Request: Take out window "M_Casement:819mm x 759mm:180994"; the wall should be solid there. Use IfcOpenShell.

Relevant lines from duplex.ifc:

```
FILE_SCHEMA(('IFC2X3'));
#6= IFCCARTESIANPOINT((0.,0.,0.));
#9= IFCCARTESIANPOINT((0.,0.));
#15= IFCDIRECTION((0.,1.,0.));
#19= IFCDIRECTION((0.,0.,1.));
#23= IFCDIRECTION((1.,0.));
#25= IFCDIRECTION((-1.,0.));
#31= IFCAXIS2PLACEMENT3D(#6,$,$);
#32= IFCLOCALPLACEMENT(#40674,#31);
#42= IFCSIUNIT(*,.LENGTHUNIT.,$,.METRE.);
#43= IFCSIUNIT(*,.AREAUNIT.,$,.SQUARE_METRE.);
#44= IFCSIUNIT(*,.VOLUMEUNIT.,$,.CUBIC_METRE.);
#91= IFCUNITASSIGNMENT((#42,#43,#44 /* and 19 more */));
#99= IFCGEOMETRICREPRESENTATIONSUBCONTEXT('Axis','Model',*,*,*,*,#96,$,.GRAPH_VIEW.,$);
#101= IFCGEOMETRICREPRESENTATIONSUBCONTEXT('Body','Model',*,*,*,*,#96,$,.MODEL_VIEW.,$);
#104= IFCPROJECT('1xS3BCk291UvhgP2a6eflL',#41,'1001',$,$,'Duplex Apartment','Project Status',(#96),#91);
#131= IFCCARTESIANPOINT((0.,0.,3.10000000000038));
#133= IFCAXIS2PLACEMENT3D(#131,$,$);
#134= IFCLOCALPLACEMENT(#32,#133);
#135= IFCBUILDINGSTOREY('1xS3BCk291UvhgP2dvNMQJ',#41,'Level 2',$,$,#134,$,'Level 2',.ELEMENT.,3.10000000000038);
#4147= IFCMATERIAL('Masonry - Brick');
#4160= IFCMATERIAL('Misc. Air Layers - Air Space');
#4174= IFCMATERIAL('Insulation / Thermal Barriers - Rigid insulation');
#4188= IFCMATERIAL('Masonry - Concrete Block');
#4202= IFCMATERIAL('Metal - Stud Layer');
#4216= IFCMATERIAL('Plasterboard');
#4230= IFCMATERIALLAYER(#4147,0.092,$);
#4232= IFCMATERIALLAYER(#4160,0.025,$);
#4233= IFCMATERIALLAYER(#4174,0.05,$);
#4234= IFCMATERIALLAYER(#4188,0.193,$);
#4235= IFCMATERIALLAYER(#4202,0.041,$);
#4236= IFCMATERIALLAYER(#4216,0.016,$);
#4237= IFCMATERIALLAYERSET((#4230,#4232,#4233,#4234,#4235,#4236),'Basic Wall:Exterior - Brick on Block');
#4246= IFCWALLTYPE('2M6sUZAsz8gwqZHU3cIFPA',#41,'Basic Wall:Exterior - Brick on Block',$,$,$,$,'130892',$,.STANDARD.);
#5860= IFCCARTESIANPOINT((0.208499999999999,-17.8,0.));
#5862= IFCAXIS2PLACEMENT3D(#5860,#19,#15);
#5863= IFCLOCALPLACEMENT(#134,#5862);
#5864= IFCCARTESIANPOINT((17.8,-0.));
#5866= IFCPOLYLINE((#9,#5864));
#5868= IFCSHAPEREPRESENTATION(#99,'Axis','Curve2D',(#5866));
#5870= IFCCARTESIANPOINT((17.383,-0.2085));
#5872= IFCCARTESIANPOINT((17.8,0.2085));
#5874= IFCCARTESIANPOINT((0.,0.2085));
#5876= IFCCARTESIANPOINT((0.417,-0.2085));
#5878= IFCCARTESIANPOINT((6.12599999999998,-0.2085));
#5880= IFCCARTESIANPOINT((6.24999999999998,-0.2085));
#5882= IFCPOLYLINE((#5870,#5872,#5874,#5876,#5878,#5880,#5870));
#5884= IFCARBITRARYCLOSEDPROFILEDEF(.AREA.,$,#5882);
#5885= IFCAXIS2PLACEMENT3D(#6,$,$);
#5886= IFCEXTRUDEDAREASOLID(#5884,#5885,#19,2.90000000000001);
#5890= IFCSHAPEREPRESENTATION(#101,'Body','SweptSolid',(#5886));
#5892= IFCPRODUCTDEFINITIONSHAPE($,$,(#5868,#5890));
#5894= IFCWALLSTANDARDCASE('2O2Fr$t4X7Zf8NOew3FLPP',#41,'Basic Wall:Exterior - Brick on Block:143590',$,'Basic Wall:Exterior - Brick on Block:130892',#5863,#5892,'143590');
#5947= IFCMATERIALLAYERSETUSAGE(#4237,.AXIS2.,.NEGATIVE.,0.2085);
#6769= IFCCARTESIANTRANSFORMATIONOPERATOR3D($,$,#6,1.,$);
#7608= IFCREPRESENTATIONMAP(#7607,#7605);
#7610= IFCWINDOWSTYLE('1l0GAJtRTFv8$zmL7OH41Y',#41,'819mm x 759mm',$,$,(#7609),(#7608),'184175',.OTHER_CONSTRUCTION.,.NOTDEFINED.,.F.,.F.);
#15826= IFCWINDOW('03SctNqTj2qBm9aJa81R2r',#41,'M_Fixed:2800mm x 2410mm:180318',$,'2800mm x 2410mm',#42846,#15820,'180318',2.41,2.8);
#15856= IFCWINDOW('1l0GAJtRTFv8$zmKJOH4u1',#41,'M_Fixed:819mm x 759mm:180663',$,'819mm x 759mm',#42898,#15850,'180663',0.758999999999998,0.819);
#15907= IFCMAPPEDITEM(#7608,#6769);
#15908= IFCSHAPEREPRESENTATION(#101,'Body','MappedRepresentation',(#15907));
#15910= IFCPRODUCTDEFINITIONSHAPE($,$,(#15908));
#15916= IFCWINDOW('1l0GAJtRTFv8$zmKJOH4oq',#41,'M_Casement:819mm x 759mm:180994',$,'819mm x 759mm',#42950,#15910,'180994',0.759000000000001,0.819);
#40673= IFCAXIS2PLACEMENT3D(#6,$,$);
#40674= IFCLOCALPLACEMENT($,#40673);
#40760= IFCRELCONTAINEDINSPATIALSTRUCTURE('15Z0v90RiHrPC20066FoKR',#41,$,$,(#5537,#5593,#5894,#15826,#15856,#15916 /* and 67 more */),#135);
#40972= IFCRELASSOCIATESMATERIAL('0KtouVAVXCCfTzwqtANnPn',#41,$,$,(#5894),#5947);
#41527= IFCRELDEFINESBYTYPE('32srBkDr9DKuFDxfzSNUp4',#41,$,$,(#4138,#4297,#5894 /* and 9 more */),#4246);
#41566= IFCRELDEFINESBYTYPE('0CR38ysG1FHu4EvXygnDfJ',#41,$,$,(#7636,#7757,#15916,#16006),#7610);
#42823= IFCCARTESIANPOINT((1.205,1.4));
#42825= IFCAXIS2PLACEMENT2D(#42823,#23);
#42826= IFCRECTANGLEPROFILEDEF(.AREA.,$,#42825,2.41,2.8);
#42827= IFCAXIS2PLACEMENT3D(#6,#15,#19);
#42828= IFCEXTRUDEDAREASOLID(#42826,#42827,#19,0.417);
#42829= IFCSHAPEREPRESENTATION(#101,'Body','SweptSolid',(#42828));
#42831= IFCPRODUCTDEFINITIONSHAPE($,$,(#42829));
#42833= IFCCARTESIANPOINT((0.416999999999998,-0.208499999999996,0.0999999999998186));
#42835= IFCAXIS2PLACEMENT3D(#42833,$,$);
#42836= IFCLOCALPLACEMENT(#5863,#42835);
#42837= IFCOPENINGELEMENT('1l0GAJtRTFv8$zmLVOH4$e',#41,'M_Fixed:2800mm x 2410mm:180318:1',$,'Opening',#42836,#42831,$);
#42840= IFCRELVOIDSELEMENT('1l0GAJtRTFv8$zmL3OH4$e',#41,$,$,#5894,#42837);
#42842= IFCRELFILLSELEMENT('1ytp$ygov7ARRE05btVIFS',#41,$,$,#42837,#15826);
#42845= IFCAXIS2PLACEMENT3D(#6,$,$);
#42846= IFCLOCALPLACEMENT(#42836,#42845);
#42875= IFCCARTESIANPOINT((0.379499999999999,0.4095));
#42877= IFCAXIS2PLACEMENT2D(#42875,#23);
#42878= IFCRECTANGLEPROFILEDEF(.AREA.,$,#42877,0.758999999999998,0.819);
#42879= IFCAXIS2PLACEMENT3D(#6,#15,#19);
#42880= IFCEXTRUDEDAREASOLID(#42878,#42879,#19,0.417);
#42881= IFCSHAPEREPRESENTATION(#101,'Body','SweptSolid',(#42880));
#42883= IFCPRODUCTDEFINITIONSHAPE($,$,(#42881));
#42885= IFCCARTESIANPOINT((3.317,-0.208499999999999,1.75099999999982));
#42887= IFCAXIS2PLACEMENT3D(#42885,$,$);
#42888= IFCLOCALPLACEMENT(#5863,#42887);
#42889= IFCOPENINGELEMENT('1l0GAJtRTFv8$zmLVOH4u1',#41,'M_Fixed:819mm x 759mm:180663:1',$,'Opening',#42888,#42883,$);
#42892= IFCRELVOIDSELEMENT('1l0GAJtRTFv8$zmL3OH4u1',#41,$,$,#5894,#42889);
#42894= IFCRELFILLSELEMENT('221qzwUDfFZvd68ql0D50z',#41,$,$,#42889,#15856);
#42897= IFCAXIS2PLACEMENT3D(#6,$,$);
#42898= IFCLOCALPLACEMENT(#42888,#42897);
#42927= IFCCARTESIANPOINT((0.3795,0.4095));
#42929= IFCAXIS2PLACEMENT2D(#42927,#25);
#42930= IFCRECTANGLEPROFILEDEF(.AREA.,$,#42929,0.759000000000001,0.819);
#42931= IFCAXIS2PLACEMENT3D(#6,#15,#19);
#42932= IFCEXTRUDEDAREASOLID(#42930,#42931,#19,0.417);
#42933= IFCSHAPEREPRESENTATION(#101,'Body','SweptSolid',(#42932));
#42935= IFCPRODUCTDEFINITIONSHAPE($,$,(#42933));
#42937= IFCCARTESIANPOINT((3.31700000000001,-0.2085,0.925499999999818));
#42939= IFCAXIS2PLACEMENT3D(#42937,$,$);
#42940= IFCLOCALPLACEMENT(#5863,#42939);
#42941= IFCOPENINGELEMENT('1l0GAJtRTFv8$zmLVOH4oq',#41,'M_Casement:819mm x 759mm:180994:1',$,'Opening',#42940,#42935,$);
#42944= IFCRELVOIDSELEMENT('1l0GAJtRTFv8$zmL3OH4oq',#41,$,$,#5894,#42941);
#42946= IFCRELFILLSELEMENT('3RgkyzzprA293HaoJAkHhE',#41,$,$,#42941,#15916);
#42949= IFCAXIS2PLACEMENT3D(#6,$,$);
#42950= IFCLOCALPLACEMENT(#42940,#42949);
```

```python
import ifcopenshell
import ifcopenshell.api.feature
import ifcopenshell.api.root
import ifcopenshell.geom
import ifcopenshell.util.shape

model = ifcopenshell.open("duplex.ifc")
settings = ifcopenshell.geom.settings()


def volume(element):
    """Net volume in cubic metres, openings subtracted."""
    shape = ifcopenshell.geom.create_shape(settings, element)
    return ifcopenshell.util.shape.get_volume(shape.geometry)


window = model.by_guid("1l0GAJtRTFv8$zmKJOH4oq")
opening = window.FillsVoids[0].RelatingOpeningElement
wall = opening.VoidsElements[0].RelatingBuildingElement
before = volume(wall)

ifcopenshell.api.root.remove_product(model, product=window)
ifcopenshell.api.feature.remove_feature(model, feature=opening)

after = volume(wall)

print(f"wall volume {before:.3f} -> {after:.3f} m3")

model.write("duplex_rev.ifc")
```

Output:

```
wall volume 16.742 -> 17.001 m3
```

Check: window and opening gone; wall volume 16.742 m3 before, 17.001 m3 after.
